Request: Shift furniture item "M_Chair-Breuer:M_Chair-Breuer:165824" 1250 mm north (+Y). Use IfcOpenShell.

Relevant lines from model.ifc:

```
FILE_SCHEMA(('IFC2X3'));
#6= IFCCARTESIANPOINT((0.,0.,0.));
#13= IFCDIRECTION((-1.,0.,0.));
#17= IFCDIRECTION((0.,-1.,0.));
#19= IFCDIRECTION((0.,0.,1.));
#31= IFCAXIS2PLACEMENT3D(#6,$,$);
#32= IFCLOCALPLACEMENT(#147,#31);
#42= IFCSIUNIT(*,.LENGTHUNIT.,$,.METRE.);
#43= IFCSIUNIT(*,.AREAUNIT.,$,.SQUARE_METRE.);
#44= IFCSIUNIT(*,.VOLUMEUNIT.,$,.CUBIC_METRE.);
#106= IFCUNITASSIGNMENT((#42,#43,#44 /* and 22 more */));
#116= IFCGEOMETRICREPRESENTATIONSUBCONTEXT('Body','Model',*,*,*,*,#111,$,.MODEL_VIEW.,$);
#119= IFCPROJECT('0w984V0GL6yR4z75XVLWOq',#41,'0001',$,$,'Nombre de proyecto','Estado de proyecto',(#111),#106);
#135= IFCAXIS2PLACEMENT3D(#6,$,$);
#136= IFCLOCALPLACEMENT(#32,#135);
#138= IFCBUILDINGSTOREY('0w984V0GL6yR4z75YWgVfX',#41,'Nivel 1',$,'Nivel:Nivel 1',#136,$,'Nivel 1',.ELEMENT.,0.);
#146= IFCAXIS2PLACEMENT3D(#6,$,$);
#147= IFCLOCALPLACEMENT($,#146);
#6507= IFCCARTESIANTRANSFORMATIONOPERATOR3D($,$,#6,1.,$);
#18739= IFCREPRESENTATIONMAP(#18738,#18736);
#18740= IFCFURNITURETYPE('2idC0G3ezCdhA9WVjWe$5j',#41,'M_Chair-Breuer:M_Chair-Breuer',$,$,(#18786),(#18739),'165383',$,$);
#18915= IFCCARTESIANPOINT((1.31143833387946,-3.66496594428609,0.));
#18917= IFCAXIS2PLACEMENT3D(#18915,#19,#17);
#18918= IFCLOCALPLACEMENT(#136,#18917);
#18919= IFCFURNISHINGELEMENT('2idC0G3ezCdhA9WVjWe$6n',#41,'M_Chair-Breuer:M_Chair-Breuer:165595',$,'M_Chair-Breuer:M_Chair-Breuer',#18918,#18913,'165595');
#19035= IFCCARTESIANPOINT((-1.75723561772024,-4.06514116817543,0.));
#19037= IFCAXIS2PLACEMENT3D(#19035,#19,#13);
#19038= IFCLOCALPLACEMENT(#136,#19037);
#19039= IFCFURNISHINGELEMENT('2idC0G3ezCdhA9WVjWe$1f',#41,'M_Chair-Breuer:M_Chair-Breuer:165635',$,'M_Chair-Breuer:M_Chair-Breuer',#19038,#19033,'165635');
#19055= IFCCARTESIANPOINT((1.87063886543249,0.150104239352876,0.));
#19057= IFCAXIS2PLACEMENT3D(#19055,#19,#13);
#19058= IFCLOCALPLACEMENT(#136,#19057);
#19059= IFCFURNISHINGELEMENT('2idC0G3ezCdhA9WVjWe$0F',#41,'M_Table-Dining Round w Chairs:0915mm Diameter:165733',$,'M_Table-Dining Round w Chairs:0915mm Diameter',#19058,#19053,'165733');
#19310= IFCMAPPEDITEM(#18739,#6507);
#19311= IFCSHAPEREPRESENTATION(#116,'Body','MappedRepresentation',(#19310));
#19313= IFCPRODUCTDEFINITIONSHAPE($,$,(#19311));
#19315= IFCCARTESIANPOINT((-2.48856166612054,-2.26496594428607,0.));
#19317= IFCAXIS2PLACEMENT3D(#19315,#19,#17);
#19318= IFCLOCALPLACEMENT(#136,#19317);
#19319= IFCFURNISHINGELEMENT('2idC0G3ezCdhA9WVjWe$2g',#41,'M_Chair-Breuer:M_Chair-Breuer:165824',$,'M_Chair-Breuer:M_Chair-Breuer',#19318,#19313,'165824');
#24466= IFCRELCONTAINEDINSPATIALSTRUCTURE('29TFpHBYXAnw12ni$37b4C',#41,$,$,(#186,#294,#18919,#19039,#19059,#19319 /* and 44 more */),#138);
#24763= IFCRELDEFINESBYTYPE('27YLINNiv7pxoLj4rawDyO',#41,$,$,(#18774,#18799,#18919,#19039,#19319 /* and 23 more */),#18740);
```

```python
import ifcopenshell
import ifcopenshell.api.geometry
import ifcopenshell.util.placement
import ifcopenshell.util.unit

model = ifcopenshell.open("model.ifc")
unit_scale = ifcopenshell.util.unit.calculate_unit_scale(model)

item = model.by_guid("2idC0G3ezCdhA9WVjWe$2g")
matrix = ifcopenshell.util.placement.get_local_placement(item.ObjectPlacement)
matrix[1, 3] += 1.25 / unit_scale
ifcopenshell.api.geometry.edit_object_placement(model, product=item, matrix=matrix, is_si=False)

print(ifcopenshell.util.placement.get_local_placement(item.ObjectPlacement).round(3) + 0.0)

model.write("model_updated.ifc")
```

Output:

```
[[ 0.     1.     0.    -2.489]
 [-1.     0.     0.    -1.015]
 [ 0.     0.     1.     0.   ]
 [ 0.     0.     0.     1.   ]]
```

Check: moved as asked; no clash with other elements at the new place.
